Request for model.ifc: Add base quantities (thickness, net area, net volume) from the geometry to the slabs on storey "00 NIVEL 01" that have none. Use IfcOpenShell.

First a look at what the model holds.

```python
import ifcopenshell
import ifcopenshell.util.element
import ifcopenshell.util.unit

model = ifcopenshell.open("model.ifc")
print(model.schema)
for unit_type in ("LENGTHUNIT", "AREAUNIT", "VOLUMEUNIT"):
    print(unit_type, ifcopenshell.util.unit.calculate_unit_scale(model, unit_type))
storey = next(s for s in model.by_type("IfcBuildingStorey") if s.Name == "00 NIVEL 01")
slabs = [e for e in ifcopenshell.util.element.get_decomposition(storey) if e.is_a("IfcSlab")]
for e in sorted(slabs, key=lambda e: e.id()):
    print(e.id(), e.is_a(), e.Name, list(ifcopenshell.util.element.get_psets(e, qtos_only=True)), sep=" | ")
```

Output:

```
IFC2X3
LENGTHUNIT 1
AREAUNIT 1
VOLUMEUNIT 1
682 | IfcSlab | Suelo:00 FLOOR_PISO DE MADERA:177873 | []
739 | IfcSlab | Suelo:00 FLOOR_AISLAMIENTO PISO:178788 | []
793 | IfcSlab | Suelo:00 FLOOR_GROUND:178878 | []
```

```python
import ifcopenshell
import ifcopenshell.api.pset
import ifcopenshell.geom
import ifcopenshell.util.element
import ifcopenshell.util.shape
import ifcopenshell.util.unit

model = ifcopenshell.open("model.ifc")
unit_scale = ifcopenshell.util.unit.calculate_unit_scale(model)
area_scale = ifcopenshell.util.unit.calculate_unit_scale(model, "AREAUNIT")
volume_scale = ifcopenshell.util.unit.calculate_unit_scale(model, "VOLUMEUNIT")
settings = ifcopenshell.geom.settings()

storey = next(s for s in model.by_type("IfcBuildingStorey") if s.Name == "00 NIVEL 01")
slabs = [e for e in ifcopenshell.util.element.get_decomposition(storey) if e.is_a("IfcSlab")]

for e in sorted(slabs, key=lambda e: e.id()):
    if ifcopenshell.util.element.get_psets(e, qtos_only=True, should_inherit=False):
        continue
    # Geometry comes back in metres, in the element's own axes.
    shape = ifcopenshell.geom.create_shape(settings, e)
    values = {
        "Width": ifcopenshell.util.shape.get_z(shape.geometry) / unit_scale,
        "NetArea": ifcopenshell.util.shape.get_footprint_area(shape.geometry) / area_scale,
        "NetVolume": ifcopenshell.util.shape.get_volume(shape.geometry) / volume_scale,
    }
    qto = ifcopenshell.api.pset.add_qto(model, product=e, name="BaseQuantities")
    ifcopenshell.api.pset.edit_qto(model, qto=qto, properties=values)
    print(e.id(), {k: round(v, 3) for k, v in values.items()})

model.write("model_edited.ifc")
```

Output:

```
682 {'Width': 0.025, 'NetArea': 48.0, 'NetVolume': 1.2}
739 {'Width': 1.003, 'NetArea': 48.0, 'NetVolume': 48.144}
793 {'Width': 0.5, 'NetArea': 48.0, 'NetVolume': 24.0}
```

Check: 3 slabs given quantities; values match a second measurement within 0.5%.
